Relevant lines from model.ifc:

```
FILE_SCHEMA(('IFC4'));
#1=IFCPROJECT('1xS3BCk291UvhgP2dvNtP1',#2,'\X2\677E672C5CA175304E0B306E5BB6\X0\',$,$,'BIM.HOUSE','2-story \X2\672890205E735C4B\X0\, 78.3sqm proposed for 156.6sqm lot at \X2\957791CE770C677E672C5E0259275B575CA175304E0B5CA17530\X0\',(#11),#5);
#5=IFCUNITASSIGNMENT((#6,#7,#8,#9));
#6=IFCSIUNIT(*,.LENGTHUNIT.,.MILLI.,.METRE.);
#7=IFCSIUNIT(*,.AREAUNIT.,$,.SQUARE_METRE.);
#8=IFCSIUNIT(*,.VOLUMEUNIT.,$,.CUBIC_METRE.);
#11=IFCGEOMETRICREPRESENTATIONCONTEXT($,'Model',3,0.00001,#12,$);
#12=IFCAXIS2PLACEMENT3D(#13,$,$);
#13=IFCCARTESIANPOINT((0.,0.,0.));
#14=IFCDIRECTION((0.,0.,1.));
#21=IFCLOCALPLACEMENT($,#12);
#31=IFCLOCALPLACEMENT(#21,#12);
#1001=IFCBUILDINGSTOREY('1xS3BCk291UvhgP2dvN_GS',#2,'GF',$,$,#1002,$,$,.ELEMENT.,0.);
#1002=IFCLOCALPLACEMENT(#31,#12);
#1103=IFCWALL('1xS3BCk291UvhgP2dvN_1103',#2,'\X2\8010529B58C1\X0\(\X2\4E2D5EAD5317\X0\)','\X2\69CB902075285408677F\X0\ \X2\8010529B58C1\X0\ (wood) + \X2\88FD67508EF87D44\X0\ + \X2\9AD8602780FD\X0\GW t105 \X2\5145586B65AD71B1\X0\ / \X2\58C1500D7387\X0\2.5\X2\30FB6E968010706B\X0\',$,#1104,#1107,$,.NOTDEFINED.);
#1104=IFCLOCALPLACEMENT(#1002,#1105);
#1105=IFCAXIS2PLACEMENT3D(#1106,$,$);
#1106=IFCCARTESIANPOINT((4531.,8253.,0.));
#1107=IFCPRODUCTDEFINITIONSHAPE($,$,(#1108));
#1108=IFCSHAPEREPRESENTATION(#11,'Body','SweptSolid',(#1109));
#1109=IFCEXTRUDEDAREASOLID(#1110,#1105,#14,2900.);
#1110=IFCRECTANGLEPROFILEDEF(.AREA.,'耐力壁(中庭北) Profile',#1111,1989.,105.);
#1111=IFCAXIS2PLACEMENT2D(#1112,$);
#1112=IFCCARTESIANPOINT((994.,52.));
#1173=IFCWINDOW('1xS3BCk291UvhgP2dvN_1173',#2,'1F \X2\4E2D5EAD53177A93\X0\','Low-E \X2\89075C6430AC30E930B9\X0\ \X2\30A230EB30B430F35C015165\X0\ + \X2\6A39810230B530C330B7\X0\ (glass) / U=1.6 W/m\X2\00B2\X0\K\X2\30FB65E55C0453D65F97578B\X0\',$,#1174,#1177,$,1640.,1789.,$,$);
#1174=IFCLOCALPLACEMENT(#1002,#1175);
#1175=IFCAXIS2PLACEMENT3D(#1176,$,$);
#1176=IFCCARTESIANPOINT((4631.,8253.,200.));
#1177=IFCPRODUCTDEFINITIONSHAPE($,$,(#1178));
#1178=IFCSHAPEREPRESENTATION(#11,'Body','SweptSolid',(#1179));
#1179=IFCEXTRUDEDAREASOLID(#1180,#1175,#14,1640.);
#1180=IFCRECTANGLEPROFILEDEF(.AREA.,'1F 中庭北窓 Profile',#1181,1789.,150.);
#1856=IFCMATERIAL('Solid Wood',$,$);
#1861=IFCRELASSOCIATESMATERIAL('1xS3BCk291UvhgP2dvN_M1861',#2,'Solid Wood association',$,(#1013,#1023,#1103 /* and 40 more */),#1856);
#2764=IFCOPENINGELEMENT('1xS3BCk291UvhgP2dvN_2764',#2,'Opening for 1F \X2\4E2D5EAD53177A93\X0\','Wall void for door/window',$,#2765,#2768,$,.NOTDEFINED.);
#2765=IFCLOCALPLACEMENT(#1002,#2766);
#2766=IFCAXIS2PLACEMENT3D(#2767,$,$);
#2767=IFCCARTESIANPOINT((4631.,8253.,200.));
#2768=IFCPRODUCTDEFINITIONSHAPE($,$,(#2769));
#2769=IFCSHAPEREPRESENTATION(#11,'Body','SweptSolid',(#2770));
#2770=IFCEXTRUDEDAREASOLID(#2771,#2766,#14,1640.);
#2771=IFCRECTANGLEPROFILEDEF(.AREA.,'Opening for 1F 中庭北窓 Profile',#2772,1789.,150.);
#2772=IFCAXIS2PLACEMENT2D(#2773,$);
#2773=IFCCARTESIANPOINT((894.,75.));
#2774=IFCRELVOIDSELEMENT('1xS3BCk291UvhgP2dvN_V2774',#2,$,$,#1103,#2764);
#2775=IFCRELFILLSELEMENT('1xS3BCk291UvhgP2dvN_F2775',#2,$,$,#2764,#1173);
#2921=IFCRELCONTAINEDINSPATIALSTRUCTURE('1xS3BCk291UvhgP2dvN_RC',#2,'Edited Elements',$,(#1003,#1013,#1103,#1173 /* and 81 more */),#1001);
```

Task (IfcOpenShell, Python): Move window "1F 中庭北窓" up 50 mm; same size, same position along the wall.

```python
import numpy as np
import ifcopenshell
import ifcopenshell.api.geometry
import ifcopenshell.util.placement
import ifcopenshell.util.unit

model = ifcopenshell.open("model.ifc")
unit_scale = ifcopenshell.util.unit.calculate_unit_scale(model)

window = model.by_guid("1xS3BCk291UvhgP2dvN_1173")
opening = window.FillsVoids[0].RelatingOpeningElement
dz = 0.05 / unit_scale

shift = np.array([0.0, 0.0, dz])
# The window is not placed relative to its opening, so move both.
for product in (opening, window):
    matrix = ifcopenshell.util.placement.get_local_placement(product.ObjectPlacement)
    matrix[:3, 3] += shift
    ifcopenshell.api.geometry.edit_object_placement(model, product=product, matrix=matrix, is_si=False)

print(f"moved by {dz * unit_scale:+.3f} m")

model.write("model_v2.ifc")
```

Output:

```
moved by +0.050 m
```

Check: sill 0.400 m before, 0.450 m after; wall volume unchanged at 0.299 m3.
